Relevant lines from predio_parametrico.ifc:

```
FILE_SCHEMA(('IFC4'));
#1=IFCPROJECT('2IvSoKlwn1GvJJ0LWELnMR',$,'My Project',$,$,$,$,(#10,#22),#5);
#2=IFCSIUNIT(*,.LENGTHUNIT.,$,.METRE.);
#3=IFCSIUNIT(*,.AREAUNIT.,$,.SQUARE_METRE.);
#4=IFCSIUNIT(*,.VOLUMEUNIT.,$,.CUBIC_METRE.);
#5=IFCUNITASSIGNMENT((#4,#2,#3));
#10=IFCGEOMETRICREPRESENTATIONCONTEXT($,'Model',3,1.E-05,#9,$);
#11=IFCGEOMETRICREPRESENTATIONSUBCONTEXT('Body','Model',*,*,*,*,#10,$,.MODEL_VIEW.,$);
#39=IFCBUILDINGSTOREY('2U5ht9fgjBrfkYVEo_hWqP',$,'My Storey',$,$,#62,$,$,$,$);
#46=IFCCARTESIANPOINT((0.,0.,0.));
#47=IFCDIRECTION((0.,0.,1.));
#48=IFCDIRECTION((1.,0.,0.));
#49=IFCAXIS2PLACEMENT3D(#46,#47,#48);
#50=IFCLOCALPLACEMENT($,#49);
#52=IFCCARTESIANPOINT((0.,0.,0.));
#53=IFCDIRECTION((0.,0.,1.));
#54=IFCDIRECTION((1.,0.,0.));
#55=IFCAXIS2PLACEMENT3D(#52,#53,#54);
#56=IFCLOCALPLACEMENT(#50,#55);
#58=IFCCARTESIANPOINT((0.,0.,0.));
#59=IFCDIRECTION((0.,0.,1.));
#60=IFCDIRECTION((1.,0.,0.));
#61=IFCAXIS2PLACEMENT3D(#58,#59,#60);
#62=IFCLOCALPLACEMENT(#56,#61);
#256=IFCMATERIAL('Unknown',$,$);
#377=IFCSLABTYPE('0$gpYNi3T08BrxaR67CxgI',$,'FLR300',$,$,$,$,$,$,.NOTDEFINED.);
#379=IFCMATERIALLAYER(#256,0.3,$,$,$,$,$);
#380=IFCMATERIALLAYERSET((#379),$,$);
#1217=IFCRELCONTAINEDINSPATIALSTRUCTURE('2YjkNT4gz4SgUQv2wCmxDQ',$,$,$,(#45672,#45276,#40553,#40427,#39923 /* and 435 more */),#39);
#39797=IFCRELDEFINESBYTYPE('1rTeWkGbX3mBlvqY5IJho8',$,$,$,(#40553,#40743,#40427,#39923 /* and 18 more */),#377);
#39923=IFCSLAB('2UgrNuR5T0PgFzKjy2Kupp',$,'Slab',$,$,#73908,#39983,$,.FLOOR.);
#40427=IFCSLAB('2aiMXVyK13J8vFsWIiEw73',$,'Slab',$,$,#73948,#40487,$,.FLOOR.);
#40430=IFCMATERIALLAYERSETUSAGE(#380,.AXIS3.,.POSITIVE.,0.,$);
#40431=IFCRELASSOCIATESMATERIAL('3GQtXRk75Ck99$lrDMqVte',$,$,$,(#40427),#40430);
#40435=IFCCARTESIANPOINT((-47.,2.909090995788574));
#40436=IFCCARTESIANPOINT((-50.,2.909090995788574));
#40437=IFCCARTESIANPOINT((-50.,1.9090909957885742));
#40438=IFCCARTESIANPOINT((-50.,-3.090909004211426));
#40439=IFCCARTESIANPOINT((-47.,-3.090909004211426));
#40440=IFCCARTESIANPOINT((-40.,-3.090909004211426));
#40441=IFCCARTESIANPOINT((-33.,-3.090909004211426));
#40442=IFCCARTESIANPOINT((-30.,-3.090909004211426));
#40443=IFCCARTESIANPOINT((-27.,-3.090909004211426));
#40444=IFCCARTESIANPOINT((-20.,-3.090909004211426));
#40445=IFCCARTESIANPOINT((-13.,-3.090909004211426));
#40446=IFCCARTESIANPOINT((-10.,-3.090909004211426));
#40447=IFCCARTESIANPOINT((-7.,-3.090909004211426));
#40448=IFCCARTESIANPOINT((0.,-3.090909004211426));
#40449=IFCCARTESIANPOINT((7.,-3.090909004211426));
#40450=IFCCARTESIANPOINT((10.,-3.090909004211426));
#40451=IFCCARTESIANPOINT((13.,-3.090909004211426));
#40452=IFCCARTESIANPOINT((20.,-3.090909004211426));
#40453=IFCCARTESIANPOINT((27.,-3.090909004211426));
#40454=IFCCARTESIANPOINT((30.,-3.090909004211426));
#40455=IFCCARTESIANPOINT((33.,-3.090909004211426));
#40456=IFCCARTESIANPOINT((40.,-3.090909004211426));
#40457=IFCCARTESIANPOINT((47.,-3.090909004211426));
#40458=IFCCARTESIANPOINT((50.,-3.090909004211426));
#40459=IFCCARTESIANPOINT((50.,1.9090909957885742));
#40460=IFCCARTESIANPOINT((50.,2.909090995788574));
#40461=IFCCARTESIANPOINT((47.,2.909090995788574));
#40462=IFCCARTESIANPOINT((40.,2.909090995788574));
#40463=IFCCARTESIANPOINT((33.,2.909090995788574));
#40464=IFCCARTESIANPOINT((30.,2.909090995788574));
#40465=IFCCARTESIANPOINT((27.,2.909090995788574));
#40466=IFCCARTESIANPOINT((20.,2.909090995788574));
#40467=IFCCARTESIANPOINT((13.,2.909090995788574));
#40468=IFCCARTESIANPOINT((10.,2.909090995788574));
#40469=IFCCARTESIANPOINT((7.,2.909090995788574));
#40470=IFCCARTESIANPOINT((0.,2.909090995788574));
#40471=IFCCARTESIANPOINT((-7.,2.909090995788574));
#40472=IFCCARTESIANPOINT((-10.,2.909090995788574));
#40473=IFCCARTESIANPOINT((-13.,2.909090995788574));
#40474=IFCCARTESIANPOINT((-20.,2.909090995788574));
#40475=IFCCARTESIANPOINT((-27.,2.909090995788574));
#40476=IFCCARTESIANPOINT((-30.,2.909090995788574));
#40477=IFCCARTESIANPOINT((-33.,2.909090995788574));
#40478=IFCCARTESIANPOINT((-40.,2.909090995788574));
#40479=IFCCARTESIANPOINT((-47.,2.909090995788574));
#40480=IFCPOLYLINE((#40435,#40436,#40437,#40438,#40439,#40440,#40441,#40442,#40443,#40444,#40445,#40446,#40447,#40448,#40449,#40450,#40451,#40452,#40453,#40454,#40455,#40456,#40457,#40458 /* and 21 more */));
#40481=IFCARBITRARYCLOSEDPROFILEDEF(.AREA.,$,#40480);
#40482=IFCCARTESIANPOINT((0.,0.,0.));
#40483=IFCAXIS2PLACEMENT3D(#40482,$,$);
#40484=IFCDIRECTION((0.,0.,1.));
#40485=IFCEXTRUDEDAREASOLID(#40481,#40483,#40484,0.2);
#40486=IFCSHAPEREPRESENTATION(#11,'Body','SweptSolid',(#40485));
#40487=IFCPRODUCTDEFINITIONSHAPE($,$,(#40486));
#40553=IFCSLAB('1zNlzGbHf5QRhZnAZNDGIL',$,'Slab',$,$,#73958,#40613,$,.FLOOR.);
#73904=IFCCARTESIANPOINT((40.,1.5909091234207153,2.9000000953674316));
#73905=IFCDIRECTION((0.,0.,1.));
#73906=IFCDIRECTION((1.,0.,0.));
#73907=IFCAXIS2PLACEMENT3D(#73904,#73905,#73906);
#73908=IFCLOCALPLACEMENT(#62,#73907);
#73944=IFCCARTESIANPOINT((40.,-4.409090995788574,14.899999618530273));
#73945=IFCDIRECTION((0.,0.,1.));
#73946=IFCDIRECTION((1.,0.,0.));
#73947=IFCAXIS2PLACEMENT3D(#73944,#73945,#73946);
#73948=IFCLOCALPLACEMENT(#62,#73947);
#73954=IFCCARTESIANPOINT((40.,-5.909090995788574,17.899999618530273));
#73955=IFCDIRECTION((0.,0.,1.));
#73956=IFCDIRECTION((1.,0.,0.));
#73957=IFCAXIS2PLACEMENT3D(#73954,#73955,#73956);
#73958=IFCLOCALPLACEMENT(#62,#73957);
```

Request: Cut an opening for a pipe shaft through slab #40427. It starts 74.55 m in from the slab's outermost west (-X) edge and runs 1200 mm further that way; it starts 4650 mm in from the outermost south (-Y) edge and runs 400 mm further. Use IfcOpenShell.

```python
import numpy as np
import ifcopenshell
import ifcopenshell.api.feature
import ifcopenshell.api.geometry
import ifcopenshell.api.root
import ifcopenshell.geom
import ifcopenshell.util.placement
import ifcopenshell.util.representation
import ifcopenshell.util.shape
import ifcopenshell.util.unit

model = ifcopenshell.open("predio_parametrico.ifc")
unit_scale = ifcopenshell.util.unit.calculate_unit_scale(model)
settings = ifcopenshell.geom.settings()


def volume(element):
    """Net volume in cubic metres, openings subtracted."""
    shape = ifcopenshell.geom.create_shape(settings, element)
    return ifcopenshell.util.shape.get_volume(shape.geometry)


slab = model.by_guid("2aiMXVyK13J8vFsWIiEw73")
before = volume(slab)

# Extent in the slab's own axes, in metres. The edges named are its -X and -Y sides.
slab_shape = ifcopenshell.geom.create_shape(settings, slab)
vertices = ifcopenshell.util.shape.get_vertices(slab_shape.geometry)
x_min, y_min, bottom = vertices.min(axis=0)
top = vertices[:, 2].max()

opening = ifcopenshell.api.root.create_entity(model, ifc_class="IfcOpeningElement", name="Pipe shaft opening", predefined_type="OPENING")
context = ifcopenshell.util.representation.get_context(model, "Model", "Body", "MODEL_VIEW")
width, depth = 1.2, 0.4
outline = [(0.0, 0.0), (width, 0.0), (width, depth), (0.0, depth), (0.0, 0.0)]
# Overshoot both faces by 50 mm so the cut is clean.
shape = ifcopenshell.api.geometry.add_slab_representation(
    model, context=context, depth=top - bottom + 0.1, polyline=outline
)
ifcopenshell.api.geometry.assign_representation(model, product=opening, representation=shape)

matrix = ifcopenshell.util.placement.get_local_placement(slab.ObjectPlacement)
matrix[:, 3] = matrix @ np.append(np.array([x_min + 74.55, y_min + 4.65, bottom - 0.05]) / unit_scale, 1.0)
ifcopenshell.api.geometry.edit_object_placement(model, product=opening, matrix=matrix, is_si=False)
ifcopenshell.api.feature.add_feature(model, feature=opening, element=slab)

after = volume(slab)

print(f"slab volume {before:.3f} -> {after:.3f} m3")

model.write("predio_parametrico_updated.ifc")
```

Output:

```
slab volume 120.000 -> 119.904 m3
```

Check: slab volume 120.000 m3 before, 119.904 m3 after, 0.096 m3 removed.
